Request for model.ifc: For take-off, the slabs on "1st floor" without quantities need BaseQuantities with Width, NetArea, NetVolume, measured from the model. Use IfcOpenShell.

First a look at what the model holds.

```python
import ifcopenshell
import ifcopenshell.util.element
import ifcopenshell.util.unit

model = ifcopenshell.open("model.ifc")
print(model.schema)
for unit_type in ("LENGTHUNIT", "AREAUNIT", "VOLUMEUNIT"):
    print(unit_type, ifcopenshell.util.unit.calculate_unit_scale(model, unit_type))
storey = next(s for s in model.by_type("IfcBuildingStorey") if s.Name == "1st floor")
slabs = [e for e in ifcopenshell.util.element.get_decomposition(storey) if e.is_a("IfcSlab")]
for e in sorted(slabs, key=lambda e: e.id()):
    print(e.id(), e.is_a(), e.Name, list(ifcopenshell.util.element.get_psets(e, qtos_only=True)), sep=" | ")
```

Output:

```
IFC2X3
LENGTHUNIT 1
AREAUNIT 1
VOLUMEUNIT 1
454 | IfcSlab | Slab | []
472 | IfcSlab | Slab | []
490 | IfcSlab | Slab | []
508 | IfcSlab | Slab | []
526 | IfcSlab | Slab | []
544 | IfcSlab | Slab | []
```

```python
import ifcopenshell
import ifcopenshell.api.pset
import ifcopenshell.geom
import ifcopenshell.util.element
import ifcopenshell.util.shape
import ifcopenshell.util.unit

model = ifcopenshell.open("model.ifc")
unit_scale = ifcopenshell.util.unit.calculate_unit_scale(model)
area_scale = ifcopenshell.util.unit.calculate_unit_scale(model, "AREAUNIT")
volume_scale = ifcopenshell.util.unit.calculate_unit_scale(model, "VOLUMEUNIT")
settings = ifcopenshell.geom.settings()

storey = next(s for s in model.by_type("IfcBuildingStorey") if s.Name == "1st floor")
slabs = [e for e in ifcopenshell.util.element.get_decomposition(storey) if e.is_a("IfcSlab")]

for e in sorted(slabs, key=lambda e: e.id()):
    if ifcopenshell.util.element.get_psets(e, qtos_only=True, should_inherit=False):
        continue
    # Geometry comes back in metres, in the element's own axes.
    shape = ifcopenshell.geom.create_shape(settings, e)
    values = {
        "Width": ifcopenshell.util.shape.get_z(shape.geometry) / unit_scale,
        "NetArea": ifcopenshell.util.shape.get_footprint_area(shape.geometry) / area_scale,
        "NetVolume": ifcopenshell.util.shape.get_volume(shape.geometry) / volume_scale,
    }
    qto = ifcopenshell.api.pset.add_qto(model, product=e, name="BaseQuantities")
    ifcopenshell.api.pset.edit_qto(model, qto=qto, properties=values)
    print(e.id(), {k: round(v, 3) for k, v in values.items()})

model.write("model-out.ifc")
```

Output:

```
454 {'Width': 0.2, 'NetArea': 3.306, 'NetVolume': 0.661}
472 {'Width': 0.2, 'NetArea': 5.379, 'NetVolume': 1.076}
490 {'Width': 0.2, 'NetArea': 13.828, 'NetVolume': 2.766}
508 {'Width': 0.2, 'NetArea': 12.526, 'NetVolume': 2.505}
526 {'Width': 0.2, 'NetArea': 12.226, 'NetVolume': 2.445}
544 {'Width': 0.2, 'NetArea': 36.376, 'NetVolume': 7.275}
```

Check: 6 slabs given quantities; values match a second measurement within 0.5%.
